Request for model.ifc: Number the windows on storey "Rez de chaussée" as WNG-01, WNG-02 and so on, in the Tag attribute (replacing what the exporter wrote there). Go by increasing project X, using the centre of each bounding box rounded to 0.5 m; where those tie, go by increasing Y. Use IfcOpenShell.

First a look at what the model holds.

```python
import ifcopenshell
import ifcopenshell.util.element
import ifcopenshell.util.placement

model = ifcopenshell.open("model.ifc")
print(model.schema)
storey = next(s for s in model.by_type("IfcBuildingStorey") if s.Name == "Rez de chaussée")
windows = [e for e in ifcopenshell.util.element.get_decomposition(storey) if e.is_a("IfcWindow")]
for e in sorted(windows, key=lambda e: e.id()):
    origin = ifcopenshell.util.placement.get_local_placement(e.ObjectPlacement)[:3, 3]
    print(e.id(), e.Tag, e.Name, origin.round(2) + 0.0, sep=" | ")
```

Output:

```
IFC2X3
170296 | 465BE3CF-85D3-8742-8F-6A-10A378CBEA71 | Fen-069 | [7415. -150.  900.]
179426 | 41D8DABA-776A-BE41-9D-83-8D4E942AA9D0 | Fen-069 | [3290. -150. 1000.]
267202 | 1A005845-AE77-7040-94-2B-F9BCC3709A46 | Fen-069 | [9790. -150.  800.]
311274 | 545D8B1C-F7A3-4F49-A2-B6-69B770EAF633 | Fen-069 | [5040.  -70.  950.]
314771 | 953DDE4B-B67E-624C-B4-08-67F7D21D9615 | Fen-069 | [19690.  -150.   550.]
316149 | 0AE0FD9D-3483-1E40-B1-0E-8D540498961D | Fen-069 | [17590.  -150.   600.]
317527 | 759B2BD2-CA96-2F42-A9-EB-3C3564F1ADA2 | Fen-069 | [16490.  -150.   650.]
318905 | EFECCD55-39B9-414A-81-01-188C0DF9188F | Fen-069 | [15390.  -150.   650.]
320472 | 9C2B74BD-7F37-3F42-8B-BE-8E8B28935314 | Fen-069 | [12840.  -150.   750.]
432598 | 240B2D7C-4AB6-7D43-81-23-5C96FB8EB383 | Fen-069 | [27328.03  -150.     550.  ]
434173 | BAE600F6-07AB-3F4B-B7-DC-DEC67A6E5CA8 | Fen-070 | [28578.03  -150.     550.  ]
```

```python
import ifcopenshell
import ifcopenshell.geom
import ifcopenshell.util.element
import ifcopenshell.util.shape

model = ifcopenshell.open("model.ifc")
settings = ifcopenshell.geom.settings()
settings.set("use-world-coords", True)


def centre(element):
    shape = ifcopenshell.geom.create_shape(settings, element)
    return ifcopenshell.util.shape.get_bbox_centroid(shape.geometry)


storey = next(s for s in model.by_type("IfcBuildingStorey") if s.Name == "Rez de chaussée")
windows = [e for e in ifcopenshell.util.element.get_decomposition(storey) if e.is_a("IfcWindow")]

# Insertion points can sit at a corner or the storey origin, so sort by the geometry (in metres).
centres = {e: centre(e) for e in windows}
windows.sort(key=lambda e: (round(centres[e][0] / 0.5), centres[e][1]))

for i, e in enumerate(windows, start=1):
    number = f"WNG-{i:02d}"
    e.Tag = number
    print(e.id(), number)

model.write("model_updated.ifc")
```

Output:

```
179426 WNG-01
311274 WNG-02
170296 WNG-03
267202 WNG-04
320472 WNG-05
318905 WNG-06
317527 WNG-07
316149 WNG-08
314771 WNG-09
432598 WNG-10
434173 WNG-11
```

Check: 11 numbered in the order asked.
